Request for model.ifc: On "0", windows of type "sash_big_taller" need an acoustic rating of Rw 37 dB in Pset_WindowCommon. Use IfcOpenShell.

First a look at what the model holds.

```python
import ifcopenshell
import ifcopenshell.util.element

model = ifcopenshell.open("model.ifc")
print(model.schema)
storey = next(s for s in model.by_type("IfcBuildingStorey") if s.Name == "0")
windows = [e for e in ifcopenshell.util.element.get_decomposition(storey) if e.is_a("IfcWindow")]
seen = {}
for e in windows:
    element_type = ifcopenshell.util.element.get_type(e)
    key = (element_type.Name if element_type != e and element_type else None, ifcopenshell.util.element.get_pset(e, "Pset_WindowCommon", "AcousticRating"))
    seen[key] = seen.get(key, 0) + 1
for (name, value), count in sorted(seen.items(), key=str):
    print(count, "x", name, "|", value)
```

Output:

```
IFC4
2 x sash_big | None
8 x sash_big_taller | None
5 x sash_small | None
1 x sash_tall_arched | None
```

```python
import ifcopenshell
import ifcopenshell.api.pset
import ifcopenshell.util.element

model = ifcopenshell.open("model.ifc")

storey = next(s for s in model.by_type("IfcBuildingStorey") if s.Name == "0")
windows = [e for e in ifcopenshell.util.element.get_decomposition(storey) if e.is_a("IfcWindow")]

count = 0
for e in windows:
    element_type = ifcopenshell.util.element.get_type(e)
    if element_type in (None, e) or element_type.Name != "sash_big_taller":
        continue
    # add_pset returns the element's existing set when there is one.
    pset = ifcopenshell.api.pset.add_pset(model, product=e, name="Pset_WindowCommon")
    ifcopenshell.api.pset.edit_pset(model, pset=pset, properties={"AcousticRating": "Rw 37 dB"})
    count += 1

print(count, "windows updated")

model.write("model_v2.ifc")
```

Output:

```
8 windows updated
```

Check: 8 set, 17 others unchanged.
